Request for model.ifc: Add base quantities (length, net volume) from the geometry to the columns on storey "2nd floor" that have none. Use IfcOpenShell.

First a look at what the model holds.

```python
import ifcopenshell
import ifcopenshell.util.element
import ifcopenshell.util.unit

model = ifcopenshell.open("model.ifc")
print(model.schema)
for unit_type in ("LENGTHUNIT", "AREAUNIT", "VOLUMEUNIT"):
    print(unit_type, ifcopenshell.util.unit.calculate_unit_scale(model, unit_type))
storey = next(s for s in model.by_type("IfcBuildingStorey") if s.Name == "2nd floor")
columns = [e for e in ifcopenshell.util.element.get_decomposition(storey) if e.is_a("IfcColumn")]
for e in sorted(columns, key=lambda e: e.id()):
    print(e.id(), e.is_a(), e.Name, list(ifcopenshell.util.element.get_psets(e, qtos_only=True)), sep=" | ")
```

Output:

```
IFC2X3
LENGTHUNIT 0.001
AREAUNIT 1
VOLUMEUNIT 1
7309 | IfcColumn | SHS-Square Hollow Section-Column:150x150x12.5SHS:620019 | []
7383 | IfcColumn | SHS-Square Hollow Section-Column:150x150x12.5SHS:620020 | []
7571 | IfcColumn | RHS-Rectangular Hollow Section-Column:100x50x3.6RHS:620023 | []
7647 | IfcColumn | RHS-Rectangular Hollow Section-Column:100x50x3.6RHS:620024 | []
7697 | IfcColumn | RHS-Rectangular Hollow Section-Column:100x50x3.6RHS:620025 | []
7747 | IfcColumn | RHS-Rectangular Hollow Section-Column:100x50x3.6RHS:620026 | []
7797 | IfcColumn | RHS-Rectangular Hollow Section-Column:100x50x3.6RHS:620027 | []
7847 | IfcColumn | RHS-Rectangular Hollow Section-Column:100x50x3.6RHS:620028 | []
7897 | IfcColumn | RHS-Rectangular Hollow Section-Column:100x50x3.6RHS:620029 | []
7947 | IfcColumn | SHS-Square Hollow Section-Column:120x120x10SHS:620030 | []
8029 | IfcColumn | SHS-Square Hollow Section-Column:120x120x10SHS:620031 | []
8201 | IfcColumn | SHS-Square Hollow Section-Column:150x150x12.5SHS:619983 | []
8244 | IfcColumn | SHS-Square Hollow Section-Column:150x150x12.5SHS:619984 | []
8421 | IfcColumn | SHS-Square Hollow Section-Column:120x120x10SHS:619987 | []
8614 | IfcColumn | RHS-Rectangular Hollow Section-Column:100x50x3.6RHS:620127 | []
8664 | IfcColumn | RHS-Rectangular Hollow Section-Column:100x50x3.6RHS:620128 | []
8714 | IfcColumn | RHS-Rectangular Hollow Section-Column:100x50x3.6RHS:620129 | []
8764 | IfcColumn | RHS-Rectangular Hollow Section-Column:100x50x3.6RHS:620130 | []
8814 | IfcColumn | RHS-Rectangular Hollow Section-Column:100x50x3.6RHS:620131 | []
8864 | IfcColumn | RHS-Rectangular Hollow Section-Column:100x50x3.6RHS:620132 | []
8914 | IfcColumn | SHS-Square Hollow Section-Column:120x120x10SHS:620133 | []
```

```python
import ifcopenshell
import ifcopenshell.api.pset
import ifcopenshell.geom
import ifcopenshell.util.element
import ifcopenshell.util.shape
import ifcopenshell.util.unit

model = ifcopenshell.open("model.ifc")
unit_scale = ifcopenshell.util.unit.calculate_unit_scale(model)
volume_scale = ifcopenshell.util.unit.calculate_unit_scale(model, "VOLUMEUNIT")
settings = ifcopenshell.geom.settings()

storey = next(s for s in model.by_type("IfcBuildingStorey") if s.Name == "2nd floor")
columns = [e for e in ifcopenshell.util.element.get_decomposition(storey) if e.is_a("IfcColumn")]

for e in sorted(columns, key=lambda e: e.id()):
    if ifcopenshell.util.element.get_psets(e, qtos_only=True, should_inherit=False):
        continue
    # Geometry comes back in metres, in the element's own axes.
    shape = ifcopenshell.geom.create_shape(settings, e)
    values = {
        "Length": ifcopenshell.util.shape.get_z(shape.geometry) / unit_scale,
        "NetVolume": ifcopenshell.util.shape.get_volume(shape.geometry) / volume_scale,
    }
    qto = ifcopenshell.api.pset.add_qto(model, product=e, name="BaseQuantities")
    ifcopenshell.api.pset.edit_qto(model, qto=qto, properties=values)
    print(e.id(), {k: round(v, 3) for k, v in values.items()})

model.write("model_v2.ifc")
```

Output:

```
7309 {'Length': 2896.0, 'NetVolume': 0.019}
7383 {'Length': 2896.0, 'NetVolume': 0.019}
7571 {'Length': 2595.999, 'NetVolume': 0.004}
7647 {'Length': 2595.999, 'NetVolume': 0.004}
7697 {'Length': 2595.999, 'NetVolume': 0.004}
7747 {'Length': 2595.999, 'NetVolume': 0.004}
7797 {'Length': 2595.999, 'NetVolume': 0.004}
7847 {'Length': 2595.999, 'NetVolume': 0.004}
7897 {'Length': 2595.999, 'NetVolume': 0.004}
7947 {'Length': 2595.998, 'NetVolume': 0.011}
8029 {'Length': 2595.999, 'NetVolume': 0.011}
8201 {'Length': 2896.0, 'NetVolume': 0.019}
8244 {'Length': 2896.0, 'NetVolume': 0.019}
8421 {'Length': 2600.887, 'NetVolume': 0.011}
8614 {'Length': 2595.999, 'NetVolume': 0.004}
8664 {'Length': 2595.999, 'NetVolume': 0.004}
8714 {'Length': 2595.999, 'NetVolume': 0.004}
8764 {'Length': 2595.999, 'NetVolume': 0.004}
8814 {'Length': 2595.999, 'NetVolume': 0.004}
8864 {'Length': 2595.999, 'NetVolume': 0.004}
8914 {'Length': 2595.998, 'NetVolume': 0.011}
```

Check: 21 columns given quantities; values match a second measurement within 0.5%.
